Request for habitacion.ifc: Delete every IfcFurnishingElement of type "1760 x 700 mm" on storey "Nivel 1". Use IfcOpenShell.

First a look at what the model holds.

```python
import ifcopenshell
import ifcopenshell.util.element

model = ifcopenshell.open("habitacion.ifc")
print(model.schema)
storey = next(s for s in model.by_type("IfcBuildingStorey") if s.Name == "Nivel 1")
furniture = [e for e in ifcopenshell.util.element.get_decomposition(storey) if e.is_a("IfcFurnishingElement")]
seen = {}
for e in furniture:
    element_type = ifcopenshell.util.element.get_type(e)
    name = element_type.Name if element_type not in (None, e) else None
    seen[name] = seen.get(name, 0) + 1
for name, count in sorted(seen.items(), key=str):
    print(count, "x", name)
```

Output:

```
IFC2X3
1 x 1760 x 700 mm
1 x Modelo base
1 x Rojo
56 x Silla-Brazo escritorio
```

```python
import ifcopenshell
import ifcopenshell.api.root
import ifcopenshell.util.element

model = ifcopenshell.open("habitacion.ifc")

storey = next(s for s in model.by_type("IfcBuildingStorey") if s.Name == "Nivel 1")
furniture = [e for e in ifcopenshell.util.element.get_decomposition(storey) if e.is_a("IfcFurnishingElement")]
targets = [e for e in furniture if (t := ifcopenshell.util.element.get_type(e)) not in (None, e) and t.Name == "1760 x 700 mm"]

for e in targets:
    ifcopenshell.api.root.remove_product(model, product=e)
print(len(targets), "removed")

model.write("habitacion_v2.ifc")
```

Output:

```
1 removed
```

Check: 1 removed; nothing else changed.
